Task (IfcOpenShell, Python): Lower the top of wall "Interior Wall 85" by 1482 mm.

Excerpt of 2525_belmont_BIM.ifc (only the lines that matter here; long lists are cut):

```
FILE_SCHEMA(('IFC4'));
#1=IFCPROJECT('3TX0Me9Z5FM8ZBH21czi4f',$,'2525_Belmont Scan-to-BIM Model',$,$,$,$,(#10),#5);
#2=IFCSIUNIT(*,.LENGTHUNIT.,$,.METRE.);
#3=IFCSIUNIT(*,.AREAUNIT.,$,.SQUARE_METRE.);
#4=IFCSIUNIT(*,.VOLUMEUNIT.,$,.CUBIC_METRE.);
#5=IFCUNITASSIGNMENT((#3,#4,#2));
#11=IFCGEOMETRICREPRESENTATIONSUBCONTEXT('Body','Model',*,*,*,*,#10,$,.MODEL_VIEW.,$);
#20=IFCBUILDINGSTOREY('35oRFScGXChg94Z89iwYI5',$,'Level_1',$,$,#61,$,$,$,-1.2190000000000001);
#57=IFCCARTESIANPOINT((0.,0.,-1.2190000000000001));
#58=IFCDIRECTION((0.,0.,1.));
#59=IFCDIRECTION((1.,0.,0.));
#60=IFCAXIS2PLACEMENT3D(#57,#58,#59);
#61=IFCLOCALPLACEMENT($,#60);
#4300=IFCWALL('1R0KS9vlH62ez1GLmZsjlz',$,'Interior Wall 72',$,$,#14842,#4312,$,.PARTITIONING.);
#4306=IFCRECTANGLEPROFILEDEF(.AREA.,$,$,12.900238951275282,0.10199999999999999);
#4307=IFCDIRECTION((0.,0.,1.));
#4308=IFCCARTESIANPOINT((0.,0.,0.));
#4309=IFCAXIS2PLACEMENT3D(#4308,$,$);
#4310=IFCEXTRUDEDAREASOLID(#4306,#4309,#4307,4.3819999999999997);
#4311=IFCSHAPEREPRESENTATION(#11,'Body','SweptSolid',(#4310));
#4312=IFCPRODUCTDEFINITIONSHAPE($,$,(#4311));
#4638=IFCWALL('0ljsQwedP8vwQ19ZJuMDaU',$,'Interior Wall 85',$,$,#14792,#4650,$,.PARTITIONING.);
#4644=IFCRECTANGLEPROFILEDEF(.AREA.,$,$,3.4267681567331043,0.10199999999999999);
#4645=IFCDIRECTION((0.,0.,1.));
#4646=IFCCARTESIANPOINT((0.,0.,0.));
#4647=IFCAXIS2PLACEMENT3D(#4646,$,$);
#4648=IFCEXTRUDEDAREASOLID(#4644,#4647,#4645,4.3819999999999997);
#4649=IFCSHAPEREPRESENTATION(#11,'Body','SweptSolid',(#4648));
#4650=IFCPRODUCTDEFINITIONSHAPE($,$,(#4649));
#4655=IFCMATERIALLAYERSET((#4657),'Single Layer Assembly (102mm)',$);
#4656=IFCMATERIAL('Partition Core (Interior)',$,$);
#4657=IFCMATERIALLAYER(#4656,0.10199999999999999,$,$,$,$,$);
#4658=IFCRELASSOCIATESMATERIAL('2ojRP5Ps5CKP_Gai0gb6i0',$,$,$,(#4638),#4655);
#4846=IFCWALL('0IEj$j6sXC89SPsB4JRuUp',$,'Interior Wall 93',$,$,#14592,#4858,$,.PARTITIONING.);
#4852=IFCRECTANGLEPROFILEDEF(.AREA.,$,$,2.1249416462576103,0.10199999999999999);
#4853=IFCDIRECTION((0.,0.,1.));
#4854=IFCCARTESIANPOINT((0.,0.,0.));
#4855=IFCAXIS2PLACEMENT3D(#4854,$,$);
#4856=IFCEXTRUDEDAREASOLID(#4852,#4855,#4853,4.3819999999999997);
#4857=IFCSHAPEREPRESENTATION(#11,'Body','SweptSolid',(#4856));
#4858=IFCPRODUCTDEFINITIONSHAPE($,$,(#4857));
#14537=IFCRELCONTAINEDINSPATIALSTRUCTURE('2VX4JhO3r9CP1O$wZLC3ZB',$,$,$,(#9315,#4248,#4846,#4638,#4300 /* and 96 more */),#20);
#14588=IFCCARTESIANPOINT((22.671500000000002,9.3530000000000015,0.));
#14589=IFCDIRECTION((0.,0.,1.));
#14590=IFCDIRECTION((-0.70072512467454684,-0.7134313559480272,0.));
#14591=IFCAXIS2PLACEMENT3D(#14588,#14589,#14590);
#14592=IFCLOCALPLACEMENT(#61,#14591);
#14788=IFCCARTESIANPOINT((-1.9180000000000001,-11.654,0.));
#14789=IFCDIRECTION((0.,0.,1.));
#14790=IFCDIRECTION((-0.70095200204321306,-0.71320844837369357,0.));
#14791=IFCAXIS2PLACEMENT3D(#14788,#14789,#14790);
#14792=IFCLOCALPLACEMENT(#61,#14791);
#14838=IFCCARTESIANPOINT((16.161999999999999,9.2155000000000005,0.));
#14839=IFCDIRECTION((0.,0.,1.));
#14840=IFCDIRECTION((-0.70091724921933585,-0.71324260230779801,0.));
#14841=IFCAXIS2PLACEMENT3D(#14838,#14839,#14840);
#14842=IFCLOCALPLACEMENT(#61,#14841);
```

```python
import ifcopenshell
import ifcopenshell.geom
import ifcopenshell.util.representation
import ifcopenshell.util.shape

model = ifcopenshell.open("2525_belmont_BIM.ifc")
settings = ifcopenshell.geom.settings()


def volume(element):
    """Net volume in cubic metres, openings subtracted."""
    shape = ifcopenshell.geom.create_shape(settings, element)
    return ifcopenshell.util.shape.get_volume(shape.geometry)


wall = model.by_guid("0ljsQwedP8vwQ19ZJuMDaU")
before = volume(wall)

body = ifcopenshell.util.representation.get_representation(wall, "Model", "Body")
solid = body.Items[0]
old_height = solid.Depth
solid.Depth -= 1.482
after = volume(wall)

print(f"height {old_height:g} -> {solid.Depth:g}, volume {before:.3f} -> {after:.3f} m3")

model.write("2525_belmont_BIM_rev.ifc")
```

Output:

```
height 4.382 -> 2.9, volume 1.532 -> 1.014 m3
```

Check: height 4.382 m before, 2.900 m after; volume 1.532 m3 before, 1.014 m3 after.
